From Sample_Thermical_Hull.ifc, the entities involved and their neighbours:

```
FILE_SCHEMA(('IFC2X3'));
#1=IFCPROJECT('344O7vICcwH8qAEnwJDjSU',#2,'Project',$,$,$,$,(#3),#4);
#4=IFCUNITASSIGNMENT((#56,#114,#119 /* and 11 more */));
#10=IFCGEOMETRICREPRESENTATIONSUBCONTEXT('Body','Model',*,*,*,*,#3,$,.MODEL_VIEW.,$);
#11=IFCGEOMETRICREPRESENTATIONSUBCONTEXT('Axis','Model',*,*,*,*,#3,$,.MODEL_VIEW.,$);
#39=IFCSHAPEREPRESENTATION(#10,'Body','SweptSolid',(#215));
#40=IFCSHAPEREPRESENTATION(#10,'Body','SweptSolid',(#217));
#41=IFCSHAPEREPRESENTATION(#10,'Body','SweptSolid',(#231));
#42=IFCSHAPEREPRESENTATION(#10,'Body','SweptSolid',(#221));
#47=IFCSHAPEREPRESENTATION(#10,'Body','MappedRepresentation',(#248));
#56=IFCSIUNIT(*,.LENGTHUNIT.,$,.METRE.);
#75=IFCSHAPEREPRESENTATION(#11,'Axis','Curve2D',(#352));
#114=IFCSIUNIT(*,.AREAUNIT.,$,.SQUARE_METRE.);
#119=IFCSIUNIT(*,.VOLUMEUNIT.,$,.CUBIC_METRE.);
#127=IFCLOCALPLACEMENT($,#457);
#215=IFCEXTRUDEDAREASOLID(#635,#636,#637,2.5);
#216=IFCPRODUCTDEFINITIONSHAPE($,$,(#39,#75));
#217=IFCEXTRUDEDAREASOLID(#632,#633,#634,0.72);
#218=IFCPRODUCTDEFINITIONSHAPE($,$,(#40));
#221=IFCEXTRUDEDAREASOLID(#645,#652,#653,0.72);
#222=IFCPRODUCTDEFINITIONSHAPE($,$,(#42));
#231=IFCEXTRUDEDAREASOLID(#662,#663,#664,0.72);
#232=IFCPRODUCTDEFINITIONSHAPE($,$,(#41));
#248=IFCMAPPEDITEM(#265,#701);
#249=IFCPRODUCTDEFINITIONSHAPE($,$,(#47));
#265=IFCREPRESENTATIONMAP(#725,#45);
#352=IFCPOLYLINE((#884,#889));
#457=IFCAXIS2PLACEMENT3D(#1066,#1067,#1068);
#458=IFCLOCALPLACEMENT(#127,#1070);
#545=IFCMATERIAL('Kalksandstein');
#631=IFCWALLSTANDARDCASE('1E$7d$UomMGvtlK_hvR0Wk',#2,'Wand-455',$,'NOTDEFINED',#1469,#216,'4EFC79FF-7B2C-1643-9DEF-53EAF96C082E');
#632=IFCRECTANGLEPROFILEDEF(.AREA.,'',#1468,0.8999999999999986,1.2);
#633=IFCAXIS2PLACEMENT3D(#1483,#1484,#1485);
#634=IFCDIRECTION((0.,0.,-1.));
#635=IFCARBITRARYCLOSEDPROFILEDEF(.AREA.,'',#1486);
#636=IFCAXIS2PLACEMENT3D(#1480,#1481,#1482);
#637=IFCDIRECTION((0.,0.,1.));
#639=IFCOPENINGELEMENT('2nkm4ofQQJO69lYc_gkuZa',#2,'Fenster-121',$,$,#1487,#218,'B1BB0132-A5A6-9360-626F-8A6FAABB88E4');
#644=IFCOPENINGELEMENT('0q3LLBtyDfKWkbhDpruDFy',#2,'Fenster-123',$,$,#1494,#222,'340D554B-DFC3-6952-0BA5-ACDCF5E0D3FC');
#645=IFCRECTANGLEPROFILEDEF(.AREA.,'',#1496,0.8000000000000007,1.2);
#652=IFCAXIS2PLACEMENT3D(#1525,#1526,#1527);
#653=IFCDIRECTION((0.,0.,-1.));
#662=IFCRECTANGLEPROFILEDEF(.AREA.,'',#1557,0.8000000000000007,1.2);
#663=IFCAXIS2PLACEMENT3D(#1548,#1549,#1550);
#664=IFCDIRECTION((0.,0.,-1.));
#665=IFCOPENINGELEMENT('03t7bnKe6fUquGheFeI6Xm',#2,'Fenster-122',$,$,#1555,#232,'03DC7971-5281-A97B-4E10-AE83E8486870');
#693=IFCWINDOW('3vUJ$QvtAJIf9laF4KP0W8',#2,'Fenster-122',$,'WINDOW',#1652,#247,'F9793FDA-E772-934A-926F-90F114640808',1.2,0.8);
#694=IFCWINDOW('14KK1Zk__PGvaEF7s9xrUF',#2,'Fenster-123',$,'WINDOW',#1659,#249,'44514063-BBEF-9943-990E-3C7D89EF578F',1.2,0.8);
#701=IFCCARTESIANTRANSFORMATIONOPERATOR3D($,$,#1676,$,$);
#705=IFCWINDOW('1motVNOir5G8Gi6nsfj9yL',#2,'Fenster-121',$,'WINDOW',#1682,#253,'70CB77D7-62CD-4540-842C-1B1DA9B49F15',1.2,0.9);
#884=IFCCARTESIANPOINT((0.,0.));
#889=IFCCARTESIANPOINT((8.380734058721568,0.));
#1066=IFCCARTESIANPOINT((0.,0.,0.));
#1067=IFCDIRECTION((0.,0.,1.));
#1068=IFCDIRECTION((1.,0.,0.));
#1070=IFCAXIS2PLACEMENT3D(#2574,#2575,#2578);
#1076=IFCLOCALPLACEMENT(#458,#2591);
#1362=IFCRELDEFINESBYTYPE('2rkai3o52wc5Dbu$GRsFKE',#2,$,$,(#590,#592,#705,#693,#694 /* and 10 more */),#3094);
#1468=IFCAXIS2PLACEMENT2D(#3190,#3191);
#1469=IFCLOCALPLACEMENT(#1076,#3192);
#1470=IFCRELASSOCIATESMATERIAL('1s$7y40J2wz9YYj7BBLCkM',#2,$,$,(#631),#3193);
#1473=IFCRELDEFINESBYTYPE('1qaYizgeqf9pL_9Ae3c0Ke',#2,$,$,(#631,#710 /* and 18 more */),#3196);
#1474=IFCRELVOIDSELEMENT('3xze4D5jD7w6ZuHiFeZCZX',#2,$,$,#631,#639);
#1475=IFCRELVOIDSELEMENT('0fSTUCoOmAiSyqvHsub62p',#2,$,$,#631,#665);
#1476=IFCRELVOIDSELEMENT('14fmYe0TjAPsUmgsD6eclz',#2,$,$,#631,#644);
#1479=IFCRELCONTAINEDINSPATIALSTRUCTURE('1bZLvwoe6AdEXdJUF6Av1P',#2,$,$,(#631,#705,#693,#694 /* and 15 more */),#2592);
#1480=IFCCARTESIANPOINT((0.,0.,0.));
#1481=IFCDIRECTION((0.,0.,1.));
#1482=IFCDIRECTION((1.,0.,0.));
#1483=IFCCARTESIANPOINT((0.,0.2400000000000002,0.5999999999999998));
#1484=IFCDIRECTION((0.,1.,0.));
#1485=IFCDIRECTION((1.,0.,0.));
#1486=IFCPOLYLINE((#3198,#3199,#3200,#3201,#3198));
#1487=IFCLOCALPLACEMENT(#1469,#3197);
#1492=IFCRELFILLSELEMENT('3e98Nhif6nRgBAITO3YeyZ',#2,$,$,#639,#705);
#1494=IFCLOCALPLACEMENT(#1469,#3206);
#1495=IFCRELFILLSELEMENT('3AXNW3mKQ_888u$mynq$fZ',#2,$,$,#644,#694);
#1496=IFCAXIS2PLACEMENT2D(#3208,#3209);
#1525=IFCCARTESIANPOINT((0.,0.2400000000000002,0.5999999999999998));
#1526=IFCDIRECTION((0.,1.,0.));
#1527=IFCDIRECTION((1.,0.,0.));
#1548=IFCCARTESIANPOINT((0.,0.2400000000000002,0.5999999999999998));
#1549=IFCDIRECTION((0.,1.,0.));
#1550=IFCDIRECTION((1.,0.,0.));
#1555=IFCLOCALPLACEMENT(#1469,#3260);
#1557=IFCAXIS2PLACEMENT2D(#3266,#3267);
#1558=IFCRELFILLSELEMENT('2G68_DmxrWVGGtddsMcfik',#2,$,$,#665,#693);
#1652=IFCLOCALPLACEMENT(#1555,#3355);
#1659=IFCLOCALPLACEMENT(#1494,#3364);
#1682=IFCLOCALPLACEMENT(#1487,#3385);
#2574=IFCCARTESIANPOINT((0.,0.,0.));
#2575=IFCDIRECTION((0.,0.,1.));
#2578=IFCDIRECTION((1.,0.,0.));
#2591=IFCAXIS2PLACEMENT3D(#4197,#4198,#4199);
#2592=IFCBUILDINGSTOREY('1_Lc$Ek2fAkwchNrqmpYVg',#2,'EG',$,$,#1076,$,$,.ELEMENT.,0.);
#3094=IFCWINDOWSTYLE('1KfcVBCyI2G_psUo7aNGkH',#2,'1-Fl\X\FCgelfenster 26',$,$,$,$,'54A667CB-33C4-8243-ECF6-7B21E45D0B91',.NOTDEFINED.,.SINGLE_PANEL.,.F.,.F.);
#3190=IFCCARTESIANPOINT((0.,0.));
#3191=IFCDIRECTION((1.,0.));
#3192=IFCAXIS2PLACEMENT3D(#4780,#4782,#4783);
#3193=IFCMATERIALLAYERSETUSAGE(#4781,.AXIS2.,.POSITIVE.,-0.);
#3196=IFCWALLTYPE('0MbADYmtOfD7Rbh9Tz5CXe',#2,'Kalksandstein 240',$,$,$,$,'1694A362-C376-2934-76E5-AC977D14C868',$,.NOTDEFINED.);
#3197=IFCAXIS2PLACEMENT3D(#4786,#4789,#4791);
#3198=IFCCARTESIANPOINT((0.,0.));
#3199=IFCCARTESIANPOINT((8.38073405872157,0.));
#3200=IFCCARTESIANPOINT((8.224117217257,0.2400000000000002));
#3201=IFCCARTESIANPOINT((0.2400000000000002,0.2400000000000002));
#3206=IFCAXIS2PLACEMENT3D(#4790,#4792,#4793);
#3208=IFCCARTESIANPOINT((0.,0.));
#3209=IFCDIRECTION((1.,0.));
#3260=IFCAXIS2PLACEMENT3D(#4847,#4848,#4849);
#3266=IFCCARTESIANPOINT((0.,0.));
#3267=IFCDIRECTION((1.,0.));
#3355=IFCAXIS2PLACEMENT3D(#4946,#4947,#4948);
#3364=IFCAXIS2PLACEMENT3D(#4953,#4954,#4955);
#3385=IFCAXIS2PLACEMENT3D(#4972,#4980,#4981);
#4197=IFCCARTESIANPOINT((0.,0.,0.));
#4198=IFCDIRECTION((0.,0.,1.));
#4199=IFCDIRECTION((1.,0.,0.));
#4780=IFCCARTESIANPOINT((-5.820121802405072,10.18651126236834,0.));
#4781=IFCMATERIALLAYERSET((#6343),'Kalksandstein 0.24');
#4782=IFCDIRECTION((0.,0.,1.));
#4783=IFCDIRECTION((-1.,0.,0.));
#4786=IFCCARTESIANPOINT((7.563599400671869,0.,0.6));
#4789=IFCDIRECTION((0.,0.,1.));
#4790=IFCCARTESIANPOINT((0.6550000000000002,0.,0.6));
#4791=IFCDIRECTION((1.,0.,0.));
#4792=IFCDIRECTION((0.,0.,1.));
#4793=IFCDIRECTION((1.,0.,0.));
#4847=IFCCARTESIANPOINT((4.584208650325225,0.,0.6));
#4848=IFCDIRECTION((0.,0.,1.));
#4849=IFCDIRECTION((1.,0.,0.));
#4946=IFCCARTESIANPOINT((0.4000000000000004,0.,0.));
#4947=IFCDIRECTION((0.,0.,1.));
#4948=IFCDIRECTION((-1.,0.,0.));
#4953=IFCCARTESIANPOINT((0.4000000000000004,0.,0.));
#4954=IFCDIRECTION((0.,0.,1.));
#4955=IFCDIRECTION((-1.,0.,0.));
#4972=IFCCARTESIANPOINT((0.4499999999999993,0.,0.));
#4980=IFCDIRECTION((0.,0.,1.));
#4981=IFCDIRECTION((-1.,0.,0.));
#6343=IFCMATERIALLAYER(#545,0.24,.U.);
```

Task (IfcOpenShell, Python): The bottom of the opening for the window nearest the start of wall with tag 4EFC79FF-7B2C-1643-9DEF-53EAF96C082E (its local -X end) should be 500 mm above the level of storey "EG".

```python
import numpy as np
import ifcopenshell
import ifcopenshell.api.geometry
import ifcopenshell.geom
import ifcopenshell.util.element
import ifcopenshell.util.placement
import ifcopenshell.util.shape
import ifcopenshell.util.unit

model = ifcopenshell.open("Sample_Thermical_Hull.ifc")
unit_scale = ifcopenshell.util.unit.calculate_unit_scale(model)

window = model.by_id(694)
opening = window.FillsVoids[0].RelatingOpeningElement
storey = ifcopenshell.util.element.get_container(window, ifc_class="IfcBuildingStorey")
level = ifcopenshell.util.placement.get_local_placement(storey.ObjectPlacement)[2, 3]

# The opening's origin need not be at the sill, so measure its lowest point.
shape = ifcopenshell.geom.create_shape(ifcopenshell.geom.settings(), opening)
bottom = ifcopenshell.util.shape.get_shape_bottom_elevation(shape, shape.geometry) / unit_scale
dz = level + 0.5 / unit_scale - bottom

shift = np.array([0.0, 0.0, dz])
# The window is placed relative to its opening, so it follows when the opening moves.
matrix = ifcopenshell.util.placement.get_local_placement(opening.ObjectPlacement)
matrix[:3, 3] += shift
ifcopenshell.api.geometry.edit_object_placement(
    model, product=opening, matrix=matrix, is_si=False, should_transform_children=True
)

print(f"moved by {dz * unit_scale:+.3f} m")

model.write("Sample_Thermical_Hull_updated.ifc")
```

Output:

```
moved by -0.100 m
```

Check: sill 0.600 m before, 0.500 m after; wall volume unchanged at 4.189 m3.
